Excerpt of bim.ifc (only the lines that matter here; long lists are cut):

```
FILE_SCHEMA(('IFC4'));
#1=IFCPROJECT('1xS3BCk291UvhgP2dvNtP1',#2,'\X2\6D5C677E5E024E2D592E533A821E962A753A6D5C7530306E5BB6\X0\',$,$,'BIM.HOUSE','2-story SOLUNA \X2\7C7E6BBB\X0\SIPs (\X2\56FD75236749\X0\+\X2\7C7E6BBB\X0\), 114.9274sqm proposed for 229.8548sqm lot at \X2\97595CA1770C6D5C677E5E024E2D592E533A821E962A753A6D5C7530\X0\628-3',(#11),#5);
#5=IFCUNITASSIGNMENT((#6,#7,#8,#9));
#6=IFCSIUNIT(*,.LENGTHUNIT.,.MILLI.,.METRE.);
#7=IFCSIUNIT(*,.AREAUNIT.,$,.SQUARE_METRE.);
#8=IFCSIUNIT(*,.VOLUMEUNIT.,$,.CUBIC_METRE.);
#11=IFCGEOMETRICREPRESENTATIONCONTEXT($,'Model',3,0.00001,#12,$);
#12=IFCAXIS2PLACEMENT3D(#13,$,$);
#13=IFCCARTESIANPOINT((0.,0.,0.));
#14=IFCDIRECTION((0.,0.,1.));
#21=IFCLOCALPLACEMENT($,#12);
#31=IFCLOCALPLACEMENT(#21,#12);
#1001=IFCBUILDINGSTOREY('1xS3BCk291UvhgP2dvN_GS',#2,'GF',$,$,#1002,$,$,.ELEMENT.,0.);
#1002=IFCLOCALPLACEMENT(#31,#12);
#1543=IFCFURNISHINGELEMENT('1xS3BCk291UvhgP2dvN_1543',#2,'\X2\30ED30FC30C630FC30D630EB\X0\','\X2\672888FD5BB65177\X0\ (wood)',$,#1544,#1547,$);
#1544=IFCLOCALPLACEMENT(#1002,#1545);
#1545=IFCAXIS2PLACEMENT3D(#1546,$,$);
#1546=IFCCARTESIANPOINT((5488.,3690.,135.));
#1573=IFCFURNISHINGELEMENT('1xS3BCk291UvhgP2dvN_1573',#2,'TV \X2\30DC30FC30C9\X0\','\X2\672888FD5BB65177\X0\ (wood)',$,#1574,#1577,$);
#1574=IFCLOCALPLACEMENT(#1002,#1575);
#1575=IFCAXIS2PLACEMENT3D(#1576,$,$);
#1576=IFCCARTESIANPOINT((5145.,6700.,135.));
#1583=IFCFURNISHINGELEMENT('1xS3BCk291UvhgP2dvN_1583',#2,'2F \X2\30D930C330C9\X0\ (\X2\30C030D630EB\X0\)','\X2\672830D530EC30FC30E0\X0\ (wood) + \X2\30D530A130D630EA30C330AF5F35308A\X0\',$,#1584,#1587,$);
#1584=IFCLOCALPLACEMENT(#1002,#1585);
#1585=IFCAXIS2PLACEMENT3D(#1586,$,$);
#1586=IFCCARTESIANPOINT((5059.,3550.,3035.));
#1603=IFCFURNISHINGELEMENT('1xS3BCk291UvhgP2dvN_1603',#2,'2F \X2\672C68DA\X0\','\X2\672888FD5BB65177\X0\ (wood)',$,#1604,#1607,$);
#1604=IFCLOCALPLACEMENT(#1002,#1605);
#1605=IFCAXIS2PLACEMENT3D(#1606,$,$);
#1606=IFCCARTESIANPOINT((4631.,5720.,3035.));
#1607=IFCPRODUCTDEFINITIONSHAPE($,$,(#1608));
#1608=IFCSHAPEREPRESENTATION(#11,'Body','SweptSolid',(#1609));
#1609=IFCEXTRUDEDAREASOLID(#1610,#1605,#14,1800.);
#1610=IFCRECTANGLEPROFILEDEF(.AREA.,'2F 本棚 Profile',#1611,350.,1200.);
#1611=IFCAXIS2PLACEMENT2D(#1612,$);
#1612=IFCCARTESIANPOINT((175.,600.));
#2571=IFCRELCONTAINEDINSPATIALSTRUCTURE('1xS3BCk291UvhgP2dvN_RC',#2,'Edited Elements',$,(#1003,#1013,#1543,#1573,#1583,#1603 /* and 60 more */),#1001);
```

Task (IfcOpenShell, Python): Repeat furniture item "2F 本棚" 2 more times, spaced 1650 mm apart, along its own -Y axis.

```python
import ifcopenshell
import ifcopenshell.api.geometry
import ifcopenshell.api.root
import ifcopenshell.util.element
import ifcopenshell.util.placement
import ifcopenshell.util.unit

model = ifcopenshell.open("bim.ifc")
unit_scale = ifcopenshell.util.unit.calculate_unit_scale(model)


def reuse_history(source, copy):
    """copy_class also copies each property set's owner history, people and application; keep the originals."""
    for rel in copy.IsDefinedBy:
        if rel.is_a("IfcRelDefinesByProperties") and (history := rel.RelatingPropertyDefinition.OwnerHistory):
            rel.RelatingPropertyDefinition.OwnerHistory = source.OwnerHistory
            ifcopenshell.util.element.remove_deep2(model, history)


source = model.by_guid("1xS3BCk291UvhgP2dvN_1603")
base = ifcopenshell.util.placement.get_local_placement(source.ObjectPlacement)
step = -base[:3, 1] * 1.65 / unit_scale

for i in range(1, 3):
    copy = ifcopenshell.api.root.copy_class(model, product=source)
    copy.Representation = ifcopenshell.util.element.copy_deep(
        model, source.Representation, exclude=["IfcGeometricRepresentationContext", "IfcRepresentationMap"]
    )
    reuse_history(source, copy)
    matrix = base.copy()
    matrix[:3, 3] += i * step
    print("added at", matrix[:3, 3].round(3) + 0.0)
    ifcopenshell.api.geometry.edit_object_placement(model, product=copy, matrix=matrix, is_si=False)

model.write("bim_updated.ifc")
```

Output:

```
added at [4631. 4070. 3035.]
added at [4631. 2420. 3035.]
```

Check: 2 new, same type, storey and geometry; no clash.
